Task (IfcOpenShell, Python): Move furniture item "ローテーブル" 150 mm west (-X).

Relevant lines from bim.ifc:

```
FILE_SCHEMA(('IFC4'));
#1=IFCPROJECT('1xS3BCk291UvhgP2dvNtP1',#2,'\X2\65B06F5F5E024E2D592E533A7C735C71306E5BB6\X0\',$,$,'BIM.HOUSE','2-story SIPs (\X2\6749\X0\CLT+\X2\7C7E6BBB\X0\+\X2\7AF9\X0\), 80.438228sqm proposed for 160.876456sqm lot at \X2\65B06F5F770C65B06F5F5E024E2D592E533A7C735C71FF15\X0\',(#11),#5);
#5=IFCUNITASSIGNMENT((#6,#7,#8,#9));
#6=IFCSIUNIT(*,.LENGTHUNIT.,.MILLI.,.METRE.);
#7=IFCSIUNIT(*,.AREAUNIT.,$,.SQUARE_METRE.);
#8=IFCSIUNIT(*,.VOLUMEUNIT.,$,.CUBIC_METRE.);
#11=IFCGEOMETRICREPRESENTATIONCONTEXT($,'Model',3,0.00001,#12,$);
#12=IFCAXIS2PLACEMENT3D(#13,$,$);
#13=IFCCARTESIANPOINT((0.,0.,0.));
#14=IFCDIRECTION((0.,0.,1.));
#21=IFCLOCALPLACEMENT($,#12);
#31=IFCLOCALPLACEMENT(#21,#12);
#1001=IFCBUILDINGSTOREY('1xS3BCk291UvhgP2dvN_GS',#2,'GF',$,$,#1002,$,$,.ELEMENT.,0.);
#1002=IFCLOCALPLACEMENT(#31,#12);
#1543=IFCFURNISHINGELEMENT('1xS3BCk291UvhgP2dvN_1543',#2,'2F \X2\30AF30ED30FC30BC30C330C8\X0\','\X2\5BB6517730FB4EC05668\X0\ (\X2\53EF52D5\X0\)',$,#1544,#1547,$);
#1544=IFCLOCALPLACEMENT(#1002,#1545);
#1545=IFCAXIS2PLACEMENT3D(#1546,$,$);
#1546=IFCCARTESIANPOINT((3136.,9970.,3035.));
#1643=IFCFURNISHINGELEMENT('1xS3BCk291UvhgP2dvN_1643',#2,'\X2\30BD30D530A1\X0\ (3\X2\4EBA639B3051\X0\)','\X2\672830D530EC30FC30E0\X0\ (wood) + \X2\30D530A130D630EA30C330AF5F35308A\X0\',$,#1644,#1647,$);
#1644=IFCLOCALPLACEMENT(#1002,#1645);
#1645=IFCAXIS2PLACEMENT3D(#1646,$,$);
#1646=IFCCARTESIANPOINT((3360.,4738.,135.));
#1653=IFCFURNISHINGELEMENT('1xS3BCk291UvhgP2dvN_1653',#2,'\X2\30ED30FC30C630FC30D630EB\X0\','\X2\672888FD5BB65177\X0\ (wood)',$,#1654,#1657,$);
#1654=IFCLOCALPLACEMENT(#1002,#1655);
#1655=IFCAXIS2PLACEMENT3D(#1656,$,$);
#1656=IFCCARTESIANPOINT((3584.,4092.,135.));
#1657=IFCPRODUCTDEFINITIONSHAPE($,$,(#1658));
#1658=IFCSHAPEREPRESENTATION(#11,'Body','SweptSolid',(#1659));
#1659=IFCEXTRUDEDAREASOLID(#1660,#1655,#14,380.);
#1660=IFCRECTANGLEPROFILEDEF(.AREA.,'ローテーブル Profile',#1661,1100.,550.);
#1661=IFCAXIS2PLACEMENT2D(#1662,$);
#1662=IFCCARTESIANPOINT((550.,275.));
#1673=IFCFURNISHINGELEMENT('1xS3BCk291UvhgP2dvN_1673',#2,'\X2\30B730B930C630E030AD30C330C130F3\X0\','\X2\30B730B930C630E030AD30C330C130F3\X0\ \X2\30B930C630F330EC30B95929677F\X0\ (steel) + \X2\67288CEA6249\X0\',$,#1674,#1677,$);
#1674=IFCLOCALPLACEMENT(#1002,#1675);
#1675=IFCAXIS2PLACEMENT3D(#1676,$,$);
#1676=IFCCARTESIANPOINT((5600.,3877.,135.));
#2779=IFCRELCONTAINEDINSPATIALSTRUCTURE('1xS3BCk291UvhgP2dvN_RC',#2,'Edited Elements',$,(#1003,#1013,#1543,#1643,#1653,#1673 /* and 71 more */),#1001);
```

```python
import ifcopenshell
import ifcopenshell.api.geometry
import ifcopenshell.util.placement
import ifcopenshell.util.unit

model = ifcopenshell.open("bim.ifc")
unit_scale = ifcopenshell.util.unit.calculate_unit_scale(model)

item = model.by_guid("1xS3BCk291UvhgP2dvN_1653")
matrix = ifcopenshell.util.placement.get_local_placement(item.ObjectPlacement)
matrix[0, 3] -= 0.15 / unit_scale
ifcopenshell.api.geometry.edit_object_placement(model, product=item, matrix=matrix, is_si=False)

print(ifcopenshell.util.placement.get_local_placement(item.ObjectPlacement).round(3) + 0.0)

model.write("bim_updated.ifc")
```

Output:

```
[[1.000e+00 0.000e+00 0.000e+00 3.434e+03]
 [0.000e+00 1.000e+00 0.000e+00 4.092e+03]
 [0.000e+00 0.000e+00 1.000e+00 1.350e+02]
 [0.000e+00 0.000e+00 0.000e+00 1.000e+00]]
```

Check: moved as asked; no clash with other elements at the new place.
